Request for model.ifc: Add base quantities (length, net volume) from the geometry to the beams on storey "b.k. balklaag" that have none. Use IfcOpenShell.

First a look at what the model holds.

```python
import ifcopenshell
import ifcopenshell.util.element
import ifcopenshell.util.unit

model = ifcopenshell.open("model.ifc")
print(model.schema)
for unit_type in ("LENGTHUNIT", "AREAUNIT", "VOLUMEUNIT"):
    print(unit_type, ifcopenshell.util.unit.calculate_unit_scale(model, unit_type))
storey = next(s for s in model.by_type("IfcBuildingStorey") if s.Name == "b.k. balklaag")
beams = [e for e in ifcopenshell.util.element.get_decomposition(storey) if e.is_a("IfcBeam")]
for e in sorted(beams, key=lambda e: e.id()):
    print(e.id(), e.is_a(), e.Name, list(ifcopenshell.util.element.get_psets(e, qtos_only=True)), sep=" | ")
```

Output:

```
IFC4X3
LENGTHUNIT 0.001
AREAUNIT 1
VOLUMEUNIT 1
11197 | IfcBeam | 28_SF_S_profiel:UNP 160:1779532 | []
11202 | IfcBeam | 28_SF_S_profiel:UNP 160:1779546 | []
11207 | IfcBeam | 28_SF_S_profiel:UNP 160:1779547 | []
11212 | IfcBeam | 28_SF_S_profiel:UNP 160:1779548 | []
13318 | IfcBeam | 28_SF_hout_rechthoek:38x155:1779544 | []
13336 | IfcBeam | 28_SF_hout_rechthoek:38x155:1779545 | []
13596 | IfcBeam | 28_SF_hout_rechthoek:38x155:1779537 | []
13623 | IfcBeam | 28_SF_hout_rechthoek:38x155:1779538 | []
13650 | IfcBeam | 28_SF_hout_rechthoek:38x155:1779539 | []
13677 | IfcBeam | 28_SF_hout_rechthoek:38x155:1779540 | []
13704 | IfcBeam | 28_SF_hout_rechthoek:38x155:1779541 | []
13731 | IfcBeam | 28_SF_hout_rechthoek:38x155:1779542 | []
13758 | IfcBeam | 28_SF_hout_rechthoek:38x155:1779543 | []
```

```python
import ifcopenshell
import ifcopenshell.api.pset
import ifcopenshell.geom
import ifcopenshell.util.element
import ifcopenshell.util.shape
import ifcopenshell.util.unit

model = ifcopenshell.open("model.ifc")
unit_scale = ifcopenshell.util.unit.calculate_unit_scale(model)
volume_scale = ifcopenshell.util.unit.calculate_unit_scale(model, "VOLUMEUNIT")
settings = ifcopenshell.geom.settings()

storey = next(s for s in model.by_type("IfcBuildingStorey") if s.Name == "b.k. balklaag")
beams = [e for e in ifcopenshell.util.element.get_decomposition(storey) if e.is_a("IfcBeam")]

for e in sorted(beams, key=lambda e: e.id()):
    if ifcopenshell.util.element.get_psets(e, qtos_only=True, should_inherit=False):
        continue
    # Geometry comes back in metres, in the element's own axes.
    shape = ifcopenshell.geom.create_shape(settings, e)
    values = {
        "Length": ifcopenshell.util.shape.get_max_xyz(shape.geometry) / unit_scale,
        "NetVolume": ifcopenshell.util.shape.get_volume(shape.geometry) / volume_scale,
    }
    qto = ifcopenshell.api.pset.add_qto(model, product=e, name="Qto_BeamBaseQuantities")
    ifcopenshell.api.pset.edit_qto(model, qto=qto, properties=values)
    print(e.id(), {k: round(v, 3) for k, v in values.items()})

model.write("model_rev.ifc")
```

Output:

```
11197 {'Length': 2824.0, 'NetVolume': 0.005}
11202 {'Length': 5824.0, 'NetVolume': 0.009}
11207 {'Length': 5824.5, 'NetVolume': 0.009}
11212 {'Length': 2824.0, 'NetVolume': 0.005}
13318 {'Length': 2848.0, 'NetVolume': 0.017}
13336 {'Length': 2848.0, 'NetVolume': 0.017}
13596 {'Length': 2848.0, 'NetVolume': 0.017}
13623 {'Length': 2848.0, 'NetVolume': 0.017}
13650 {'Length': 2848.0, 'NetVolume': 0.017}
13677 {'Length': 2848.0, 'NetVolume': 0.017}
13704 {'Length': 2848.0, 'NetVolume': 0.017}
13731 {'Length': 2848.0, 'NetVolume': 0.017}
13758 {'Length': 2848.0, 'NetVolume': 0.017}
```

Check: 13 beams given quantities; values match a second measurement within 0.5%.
